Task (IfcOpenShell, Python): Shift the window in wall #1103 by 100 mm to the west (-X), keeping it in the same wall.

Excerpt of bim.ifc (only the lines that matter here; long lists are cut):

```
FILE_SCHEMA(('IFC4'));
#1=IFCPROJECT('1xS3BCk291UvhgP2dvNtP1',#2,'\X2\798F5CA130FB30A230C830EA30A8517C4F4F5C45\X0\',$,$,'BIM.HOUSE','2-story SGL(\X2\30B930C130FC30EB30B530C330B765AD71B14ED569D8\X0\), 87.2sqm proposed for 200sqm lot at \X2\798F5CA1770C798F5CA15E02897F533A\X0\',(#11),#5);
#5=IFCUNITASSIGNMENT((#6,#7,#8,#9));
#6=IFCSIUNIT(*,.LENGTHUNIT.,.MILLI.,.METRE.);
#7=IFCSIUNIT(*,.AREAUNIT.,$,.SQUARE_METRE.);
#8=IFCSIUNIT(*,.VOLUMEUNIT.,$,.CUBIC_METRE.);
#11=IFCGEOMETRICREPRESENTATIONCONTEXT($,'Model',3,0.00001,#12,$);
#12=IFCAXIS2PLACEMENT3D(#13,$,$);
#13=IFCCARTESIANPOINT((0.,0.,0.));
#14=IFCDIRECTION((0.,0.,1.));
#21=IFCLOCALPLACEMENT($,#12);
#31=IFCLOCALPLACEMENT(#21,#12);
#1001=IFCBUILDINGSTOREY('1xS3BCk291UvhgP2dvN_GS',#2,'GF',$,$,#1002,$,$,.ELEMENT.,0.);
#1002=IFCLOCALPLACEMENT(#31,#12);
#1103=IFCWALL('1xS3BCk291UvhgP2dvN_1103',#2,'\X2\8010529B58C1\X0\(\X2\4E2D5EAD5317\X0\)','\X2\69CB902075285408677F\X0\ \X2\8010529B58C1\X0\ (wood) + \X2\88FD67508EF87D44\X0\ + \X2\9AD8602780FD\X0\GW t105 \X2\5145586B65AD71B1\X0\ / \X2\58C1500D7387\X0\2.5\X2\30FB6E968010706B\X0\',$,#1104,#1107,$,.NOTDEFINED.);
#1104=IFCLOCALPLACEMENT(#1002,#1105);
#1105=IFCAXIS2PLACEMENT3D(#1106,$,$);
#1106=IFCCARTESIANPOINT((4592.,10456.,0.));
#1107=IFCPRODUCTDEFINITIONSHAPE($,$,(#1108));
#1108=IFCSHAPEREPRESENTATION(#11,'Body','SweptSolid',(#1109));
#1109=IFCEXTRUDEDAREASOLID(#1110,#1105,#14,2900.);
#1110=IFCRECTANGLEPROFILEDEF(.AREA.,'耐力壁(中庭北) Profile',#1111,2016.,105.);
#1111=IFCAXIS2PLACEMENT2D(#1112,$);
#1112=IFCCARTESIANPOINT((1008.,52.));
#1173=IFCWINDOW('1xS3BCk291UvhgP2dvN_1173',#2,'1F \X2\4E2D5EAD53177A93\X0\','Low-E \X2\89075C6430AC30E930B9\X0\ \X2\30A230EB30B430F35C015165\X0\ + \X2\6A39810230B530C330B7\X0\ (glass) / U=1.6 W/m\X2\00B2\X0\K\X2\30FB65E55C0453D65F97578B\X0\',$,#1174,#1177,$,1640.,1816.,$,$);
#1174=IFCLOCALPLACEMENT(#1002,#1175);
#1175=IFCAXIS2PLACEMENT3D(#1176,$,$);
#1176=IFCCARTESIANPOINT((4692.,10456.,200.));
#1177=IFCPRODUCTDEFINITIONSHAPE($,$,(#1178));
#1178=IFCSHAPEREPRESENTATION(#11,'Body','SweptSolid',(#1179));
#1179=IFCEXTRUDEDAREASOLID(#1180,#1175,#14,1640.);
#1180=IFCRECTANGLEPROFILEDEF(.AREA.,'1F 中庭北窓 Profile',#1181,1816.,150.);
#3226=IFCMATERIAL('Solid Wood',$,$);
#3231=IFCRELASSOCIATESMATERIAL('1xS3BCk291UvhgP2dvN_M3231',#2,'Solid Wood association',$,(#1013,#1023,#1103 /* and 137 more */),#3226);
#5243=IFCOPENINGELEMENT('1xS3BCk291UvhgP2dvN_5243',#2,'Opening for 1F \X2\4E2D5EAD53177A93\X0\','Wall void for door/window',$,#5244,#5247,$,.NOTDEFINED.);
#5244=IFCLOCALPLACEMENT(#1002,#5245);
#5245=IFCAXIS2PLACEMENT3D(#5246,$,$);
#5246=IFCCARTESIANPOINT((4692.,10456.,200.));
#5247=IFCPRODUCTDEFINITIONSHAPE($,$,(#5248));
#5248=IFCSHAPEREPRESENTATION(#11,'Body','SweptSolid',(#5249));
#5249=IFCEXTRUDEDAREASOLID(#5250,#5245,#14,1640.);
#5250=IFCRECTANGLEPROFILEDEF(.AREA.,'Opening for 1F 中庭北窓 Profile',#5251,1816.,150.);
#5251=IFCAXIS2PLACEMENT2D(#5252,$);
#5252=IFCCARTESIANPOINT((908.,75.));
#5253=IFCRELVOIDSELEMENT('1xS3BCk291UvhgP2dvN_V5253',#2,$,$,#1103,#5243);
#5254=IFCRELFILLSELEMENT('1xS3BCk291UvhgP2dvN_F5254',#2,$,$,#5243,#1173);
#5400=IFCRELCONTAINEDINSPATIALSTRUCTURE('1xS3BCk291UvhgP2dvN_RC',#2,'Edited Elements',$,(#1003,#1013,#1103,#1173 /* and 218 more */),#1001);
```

```python
import ifcopenshell
import ifcopenshell.api.geometry
import ifcopenshell.util.placement

model = ifcopenshell.open("bim.ifc")

window = model.by_id(1173)
opening = window.FillsVoids[0].RelatingOpeningElement
wall = opening.VoidsElements[0].RelatingBuildingElement

wall_matrix = ifcopenshell.util.placement.get_local_placement(wall.ObjectPlacement)
shift = wall_matrix[:3, 0] * -100.0
before = ifcopenshell.util.placement.get_local_placement(window.ObjectPlacement)[:3, 3].copy()

# The window is not placed relative to its opening, so move both.
for product in (opening, window):
    matrix = ifcopenshell.util.placement.get_local_placement(product.ObjectPlacement)
    matrix[:3, 3] += shift
    ifcopenshell.api.geometry.edit_object_placement(model, product=product, matrix=matrix, is_si=False)

after = ifcopenshell.util.placement.get_local_placement(window.ObjectPlacement)[:3, 3]
print("window moved by", (after - before).round(3) + 0.0)

model.write("bim_edited.ifc")
```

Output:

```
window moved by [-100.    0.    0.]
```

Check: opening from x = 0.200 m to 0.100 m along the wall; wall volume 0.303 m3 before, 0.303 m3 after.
